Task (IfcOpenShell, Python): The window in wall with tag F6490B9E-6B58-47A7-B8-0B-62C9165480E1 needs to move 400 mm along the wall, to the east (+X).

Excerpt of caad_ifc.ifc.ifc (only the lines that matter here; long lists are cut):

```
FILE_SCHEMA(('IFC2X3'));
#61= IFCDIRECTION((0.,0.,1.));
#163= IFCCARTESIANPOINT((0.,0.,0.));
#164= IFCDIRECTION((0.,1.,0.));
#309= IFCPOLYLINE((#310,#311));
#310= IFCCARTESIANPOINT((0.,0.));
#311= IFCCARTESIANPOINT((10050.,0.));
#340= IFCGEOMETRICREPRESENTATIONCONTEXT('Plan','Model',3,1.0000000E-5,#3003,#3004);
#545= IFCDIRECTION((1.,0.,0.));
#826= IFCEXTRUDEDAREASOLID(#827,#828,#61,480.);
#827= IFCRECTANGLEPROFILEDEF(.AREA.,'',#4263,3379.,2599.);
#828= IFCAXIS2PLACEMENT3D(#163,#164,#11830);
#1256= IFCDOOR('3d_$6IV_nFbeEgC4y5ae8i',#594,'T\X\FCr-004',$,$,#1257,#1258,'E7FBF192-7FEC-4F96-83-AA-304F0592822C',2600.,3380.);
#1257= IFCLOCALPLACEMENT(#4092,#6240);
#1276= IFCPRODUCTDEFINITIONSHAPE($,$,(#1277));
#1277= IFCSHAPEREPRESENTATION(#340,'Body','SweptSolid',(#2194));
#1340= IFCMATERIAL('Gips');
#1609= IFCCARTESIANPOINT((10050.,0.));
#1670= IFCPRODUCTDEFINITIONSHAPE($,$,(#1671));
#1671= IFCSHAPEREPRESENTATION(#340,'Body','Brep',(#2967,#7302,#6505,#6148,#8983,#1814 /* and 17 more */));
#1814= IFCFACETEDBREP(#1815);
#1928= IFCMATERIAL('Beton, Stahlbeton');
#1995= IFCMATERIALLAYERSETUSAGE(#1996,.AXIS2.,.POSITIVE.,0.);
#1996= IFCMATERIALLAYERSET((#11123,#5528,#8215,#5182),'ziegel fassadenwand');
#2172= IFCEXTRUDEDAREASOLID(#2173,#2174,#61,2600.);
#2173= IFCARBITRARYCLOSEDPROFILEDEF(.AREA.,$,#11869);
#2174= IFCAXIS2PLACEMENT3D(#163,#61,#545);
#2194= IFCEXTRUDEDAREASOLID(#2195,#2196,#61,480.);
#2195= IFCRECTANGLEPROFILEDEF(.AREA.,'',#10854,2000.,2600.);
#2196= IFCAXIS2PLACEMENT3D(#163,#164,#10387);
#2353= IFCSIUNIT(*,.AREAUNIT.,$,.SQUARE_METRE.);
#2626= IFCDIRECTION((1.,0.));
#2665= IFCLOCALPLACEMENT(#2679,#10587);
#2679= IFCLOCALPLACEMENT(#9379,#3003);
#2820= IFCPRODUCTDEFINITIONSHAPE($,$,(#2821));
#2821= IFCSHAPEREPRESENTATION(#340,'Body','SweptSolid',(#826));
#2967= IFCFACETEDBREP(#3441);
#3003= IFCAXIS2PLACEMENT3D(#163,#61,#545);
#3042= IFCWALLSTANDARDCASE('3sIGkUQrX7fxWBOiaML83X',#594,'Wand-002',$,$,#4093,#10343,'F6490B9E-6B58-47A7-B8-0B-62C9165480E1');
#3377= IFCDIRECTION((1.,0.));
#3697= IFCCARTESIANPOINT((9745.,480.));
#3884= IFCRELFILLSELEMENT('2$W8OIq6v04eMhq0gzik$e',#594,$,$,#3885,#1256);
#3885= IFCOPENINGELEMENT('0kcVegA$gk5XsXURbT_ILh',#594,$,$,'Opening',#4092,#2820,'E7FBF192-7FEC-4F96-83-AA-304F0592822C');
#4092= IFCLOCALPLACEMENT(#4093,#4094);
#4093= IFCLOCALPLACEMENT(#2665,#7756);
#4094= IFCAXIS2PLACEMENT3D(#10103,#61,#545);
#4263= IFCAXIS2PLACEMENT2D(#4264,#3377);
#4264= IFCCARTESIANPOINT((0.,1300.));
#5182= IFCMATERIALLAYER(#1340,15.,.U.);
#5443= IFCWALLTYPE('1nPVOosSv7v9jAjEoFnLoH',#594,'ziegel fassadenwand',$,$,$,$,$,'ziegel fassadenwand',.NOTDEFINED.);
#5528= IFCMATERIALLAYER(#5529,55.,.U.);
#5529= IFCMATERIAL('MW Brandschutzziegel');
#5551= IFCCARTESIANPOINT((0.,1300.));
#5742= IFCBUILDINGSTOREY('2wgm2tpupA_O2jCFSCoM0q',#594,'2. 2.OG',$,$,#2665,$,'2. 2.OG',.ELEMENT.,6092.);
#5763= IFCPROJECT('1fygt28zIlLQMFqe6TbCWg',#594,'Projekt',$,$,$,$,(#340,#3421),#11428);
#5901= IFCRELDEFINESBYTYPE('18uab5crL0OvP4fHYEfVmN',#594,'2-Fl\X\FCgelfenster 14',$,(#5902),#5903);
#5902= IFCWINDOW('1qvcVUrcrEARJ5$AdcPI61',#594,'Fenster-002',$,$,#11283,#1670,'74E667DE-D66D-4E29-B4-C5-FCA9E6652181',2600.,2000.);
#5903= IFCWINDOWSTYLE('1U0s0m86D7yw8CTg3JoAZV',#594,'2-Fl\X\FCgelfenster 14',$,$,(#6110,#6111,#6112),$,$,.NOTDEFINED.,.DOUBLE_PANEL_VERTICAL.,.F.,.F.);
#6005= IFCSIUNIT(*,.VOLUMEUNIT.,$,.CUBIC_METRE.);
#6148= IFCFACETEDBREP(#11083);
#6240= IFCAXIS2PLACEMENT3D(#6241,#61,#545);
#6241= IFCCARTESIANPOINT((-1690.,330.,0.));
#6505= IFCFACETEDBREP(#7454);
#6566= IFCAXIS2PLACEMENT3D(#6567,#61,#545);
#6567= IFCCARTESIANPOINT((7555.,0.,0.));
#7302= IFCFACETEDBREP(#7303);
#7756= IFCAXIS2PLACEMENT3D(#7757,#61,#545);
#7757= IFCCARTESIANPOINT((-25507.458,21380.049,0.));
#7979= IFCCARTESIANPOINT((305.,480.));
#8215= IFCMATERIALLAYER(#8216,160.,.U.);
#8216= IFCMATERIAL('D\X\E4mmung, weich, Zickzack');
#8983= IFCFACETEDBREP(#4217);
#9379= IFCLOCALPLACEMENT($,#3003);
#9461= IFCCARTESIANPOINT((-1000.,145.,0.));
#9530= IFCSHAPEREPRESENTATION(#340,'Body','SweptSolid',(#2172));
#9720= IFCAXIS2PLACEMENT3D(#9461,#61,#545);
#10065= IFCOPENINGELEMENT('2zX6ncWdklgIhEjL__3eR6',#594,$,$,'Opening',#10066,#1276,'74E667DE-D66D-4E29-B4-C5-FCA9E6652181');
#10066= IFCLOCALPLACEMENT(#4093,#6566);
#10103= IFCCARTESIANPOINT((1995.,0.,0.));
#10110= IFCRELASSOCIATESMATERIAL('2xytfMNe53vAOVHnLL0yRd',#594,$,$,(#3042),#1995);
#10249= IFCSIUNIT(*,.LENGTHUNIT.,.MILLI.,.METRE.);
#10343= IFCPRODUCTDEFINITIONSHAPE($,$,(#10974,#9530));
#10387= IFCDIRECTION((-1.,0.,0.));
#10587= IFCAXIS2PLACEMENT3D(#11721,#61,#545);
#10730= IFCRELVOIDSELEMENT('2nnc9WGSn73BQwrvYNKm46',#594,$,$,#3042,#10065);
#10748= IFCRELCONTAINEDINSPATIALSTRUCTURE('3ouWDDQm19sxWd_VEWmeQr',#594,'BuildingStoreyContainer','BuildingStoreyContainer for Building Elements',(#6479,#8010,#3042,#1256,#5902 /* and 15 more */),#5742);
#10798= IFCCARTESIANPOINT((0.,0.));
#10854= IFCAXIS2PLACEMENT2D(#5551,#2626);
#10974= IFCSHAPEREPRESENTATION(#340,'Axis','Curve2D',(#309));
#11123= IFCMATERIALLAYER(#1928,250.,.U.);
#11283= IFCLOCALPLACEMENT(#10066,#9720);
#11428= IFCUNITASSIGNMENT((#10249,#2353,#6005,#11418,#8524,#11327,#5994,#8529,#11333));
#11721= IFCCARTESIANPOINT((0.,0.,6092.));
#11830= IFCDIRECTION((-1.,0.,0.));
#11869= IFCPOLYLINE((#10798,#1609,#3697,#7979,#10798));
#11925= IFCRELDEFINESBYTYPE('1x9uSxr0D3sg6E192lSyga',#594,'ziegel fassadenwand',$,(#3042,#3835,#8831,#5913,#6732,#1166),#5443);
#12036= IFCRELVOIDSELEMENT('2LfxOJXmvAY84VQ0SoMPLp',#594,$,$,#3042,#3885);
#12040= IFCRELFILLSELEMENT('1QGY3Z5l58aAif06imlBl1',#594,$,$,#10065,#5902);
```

```python
import ifcopenshell
import ifcopenshell.api.geometry
import ifcopenshell.util.placement
import ifcopenshell.util.unit

model = ifcopenshell.open("caad_ifc.ifc.ifc")
unit_scale = ifcopenshell.util.unit.calculate_unit_scale(model)

window = model.by_guid("1qvcVUrcrEARJ5$AdcPI61")
opening = window.FillsVoids[0].RelatingOpeningElement
wall = opening.VoidsElements[0].RelatingBuildingElement

wall_matrix = ifcopenshell.util.placement.get_local_placement(wall.ObjectPlacement)
shift = wall_matrix[:3, 0] * 0.4 / unit_scale
before = ifcopenshell.util.placement.get_local_placement(window.ObjectPlacement)[:3, 3].copy()

# The window is placed relative to its opening, so it follows when the opening moves.
matrix = ifcopenshell.util.placement.get_local_placement(opening.ObjectPlacement)
matrix[:3, 3] += shift
ifcopenshell.api.geometry.edit_object_placement(
    model, product=opening, matrix=matrix, is_si=False, should_transform_children=True
)

after = ifcopenshell.util.placement.get_local_placement(window.ObjectPlacement)[:3, 3]
print("window moved by", (after - before).round(3) + 0.0)

model.write("caad_ifc.ifc_updated.ifc")
```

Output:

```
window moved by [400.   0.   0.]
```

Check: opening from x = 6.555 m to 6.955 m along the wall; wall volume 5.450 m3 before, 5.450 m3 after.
